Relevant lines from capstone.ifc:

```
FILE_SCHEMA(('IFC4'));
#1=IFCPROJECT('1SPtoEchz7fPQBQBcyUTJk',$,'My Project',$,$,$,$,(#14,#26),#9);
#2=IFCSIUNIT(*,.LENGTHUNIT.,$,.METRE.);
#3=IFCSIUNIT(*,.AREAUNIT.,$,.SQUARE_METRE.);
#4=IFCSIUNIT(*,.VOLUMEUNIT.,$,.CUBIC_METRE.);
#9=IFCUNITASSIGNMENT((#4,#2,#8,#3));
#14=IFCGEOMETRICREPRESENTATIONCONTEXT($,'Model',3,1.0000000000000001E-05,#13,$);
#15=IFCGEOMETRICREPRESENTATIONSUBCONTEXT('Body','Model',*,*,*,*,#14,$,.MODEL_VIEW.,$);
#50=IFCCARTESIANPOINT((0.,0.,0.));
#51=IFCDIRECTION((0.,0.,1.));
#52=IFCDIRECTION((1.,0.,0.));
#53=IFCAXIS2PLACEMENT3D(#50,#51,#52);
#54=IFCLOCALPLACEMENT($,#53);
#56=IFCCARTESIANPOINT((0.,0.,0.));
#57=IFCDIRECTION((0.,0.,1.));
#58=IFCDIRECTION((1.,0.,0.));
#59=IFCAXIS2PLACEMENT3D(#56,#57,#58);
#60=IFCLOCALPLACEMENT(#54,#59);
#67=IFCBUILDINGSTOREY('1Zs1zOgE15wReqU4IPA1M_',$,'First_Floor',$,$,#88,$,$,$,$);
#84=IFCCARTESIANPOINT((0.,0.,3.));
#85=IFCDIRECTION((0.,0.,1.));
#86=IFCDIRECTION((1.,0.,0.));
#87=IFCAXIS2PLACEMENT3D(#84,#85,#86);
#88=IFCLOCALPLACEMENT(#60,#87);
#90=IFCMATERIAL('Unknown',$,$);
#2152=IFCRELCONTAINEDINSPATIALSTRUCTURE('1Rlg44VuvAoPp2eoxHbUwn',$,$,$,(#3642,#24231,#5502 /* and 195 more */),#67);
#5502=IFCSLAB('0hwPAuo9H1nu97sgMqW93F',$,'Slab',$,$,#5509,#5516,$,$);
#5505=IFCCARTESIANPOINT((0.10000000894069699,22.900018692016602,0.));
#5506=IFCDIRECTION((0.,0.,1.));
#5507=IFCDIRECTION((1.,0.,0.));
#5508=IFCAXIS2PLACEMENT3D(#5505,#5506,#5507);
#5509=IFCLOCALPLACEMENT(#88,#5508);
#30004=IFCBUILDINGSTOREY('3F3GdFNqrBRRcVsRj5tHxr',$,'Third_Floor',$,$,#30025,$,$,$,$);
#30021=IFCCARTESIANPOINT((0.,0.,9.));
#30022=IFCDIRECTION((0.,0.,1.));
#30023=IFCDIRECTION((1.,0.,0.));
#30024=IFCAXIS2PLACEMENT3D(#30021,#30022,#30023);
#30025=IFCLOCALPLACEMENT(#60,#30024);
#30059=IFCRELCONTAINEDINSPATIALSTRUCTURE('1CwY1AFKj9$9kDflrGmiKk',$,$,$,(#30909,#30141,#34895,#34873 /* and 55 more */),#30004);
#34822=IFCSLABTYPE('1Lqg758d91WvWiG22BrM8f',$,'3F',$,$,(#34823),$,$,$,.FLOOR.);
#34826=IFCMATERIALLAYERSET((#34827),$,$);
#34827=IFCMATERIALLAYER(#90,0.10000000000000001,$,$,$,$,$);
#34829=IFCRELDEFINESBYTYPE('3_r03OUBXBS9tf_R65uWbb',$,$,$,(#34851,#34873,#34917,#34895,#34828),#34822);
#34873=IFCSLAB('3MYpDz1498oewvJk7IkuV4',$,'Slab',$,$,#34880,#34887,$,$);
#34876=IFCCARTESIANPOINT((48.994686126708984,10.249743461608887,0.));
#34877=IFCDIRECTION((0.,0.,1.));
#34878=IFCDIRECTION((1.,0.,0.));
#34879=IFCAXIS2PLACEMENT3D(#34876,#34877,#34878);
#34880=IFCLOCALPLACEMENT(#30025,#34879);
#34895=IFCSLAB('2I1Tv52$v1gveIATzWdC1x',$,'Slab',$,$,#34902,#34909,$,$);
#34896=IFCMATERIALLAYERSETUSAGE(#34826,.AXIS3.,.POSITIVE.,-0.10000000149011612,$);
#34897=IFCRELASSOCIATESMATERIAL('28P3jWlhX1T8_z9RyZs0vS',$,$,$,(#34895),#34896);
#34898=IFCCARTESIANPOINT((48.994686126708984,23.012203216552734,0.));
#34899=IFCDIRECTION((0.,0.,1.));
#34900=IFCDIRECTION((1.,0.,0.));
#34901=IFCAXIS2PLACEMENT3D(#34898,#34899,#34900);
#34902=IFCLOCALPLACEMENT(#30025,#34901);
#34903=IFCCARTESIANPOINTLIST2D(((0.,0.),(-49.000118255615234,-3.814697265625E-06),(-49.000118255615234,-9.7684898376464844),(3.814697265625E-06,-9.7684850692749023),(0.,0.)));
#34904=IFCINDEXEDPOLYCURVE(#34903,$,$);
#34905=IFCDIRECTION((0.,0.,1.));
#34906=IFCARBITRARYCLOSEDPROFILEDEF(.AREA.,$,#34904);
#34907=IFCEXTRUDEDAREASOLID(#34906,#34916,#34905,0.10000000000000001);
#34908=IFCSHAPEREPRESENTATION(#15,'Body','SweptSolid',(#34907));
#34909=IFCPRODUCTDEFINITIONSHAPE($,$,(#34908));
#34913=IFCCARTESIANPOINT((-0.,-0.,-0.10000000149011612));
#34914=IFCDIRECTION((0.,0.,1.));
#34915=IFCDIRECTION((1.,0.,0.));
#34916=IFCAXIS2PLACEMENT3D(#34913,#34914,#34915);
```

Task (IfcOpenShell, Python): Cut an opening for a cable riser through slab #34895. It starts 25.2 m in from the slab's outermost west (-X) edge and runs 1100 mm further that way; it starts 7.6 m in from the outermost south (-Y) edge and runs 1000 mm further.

```python
import numpy as np
import ifcopenshell
import ifcopenshell.api.feature
import ifcopenshell.api.geometry
import ifcopenshell.api.root
import ifcopenshell.geom
import ifcopenshell.util.placement
import ifcopenshell.util.representation
import ifcopenshell.util.shape
import ifcopenshell.util.unit

model = ifcopenshell.open("capstone.ifc")
unit_scale = ifcopenshell.util.unit.calculate_unit_scale(model)
settings = ifcopenshell.geom.settings()


def volume(element):
    """Net volume in cubic metres, openings subtracted."""
    shape = ifcopenshell.geom.create_shape(settings, element)
    return ifcopenshell.util.shape.get_volume(shape.geometry)


slab = model.by_guid("2I1Tv52$v1gveIATzWdC1x")
before = volume(slab)

# Extent in the slab's own axes, in metres. The edges named are its -X and -Y sides.
slab_shape = ifcopenshell.geom.create_shape(settings, slab)
vertices = ifcopenshell.util.shape.get_vertices(slab_shape.geometry)
x_min, y_min, bottom = vertices.min(axis=0)
top = vertices[:, 2].max()

opening = ifcopenshell.api.root.create_entity(model, ifc_class="IfcOpeningElement", name="Cable riser opening", predefined_type="OPENING")
context = ifcopenshell.util.representation.get_context(model, "Model", "Body", "MODEL_VIEW")
width, depth = 1.1, 1
outline = [(0.0, 0.0), (width, 0.0), (width, depth), (0.0, depth), (0.0, 0.0)]
# Overshoot both faces by 50 mm so the cut is clean.
shape = ifcopenshell.api.geometry.add_slab_representation(
    model, context=context, depth=top - bottom + 0.1, polyline=outline
)
ifcopenshell.api.geometry.assign_representation(model, product=opening, representation=shape)

matrix = ifcopenshell.util.placement.get_local_placement(slab.ObjectPlacement)
matrix[:, 3] = matrix @ np.append(np.array([x_min + 25.2, y_min + 7.6, bottom - 0.05]) / unit_scale, 1.0)
ifcopenshell.api.geometry.edit_object_placement(model, product=opening, matrix=matrix, is_si=False)
ifcopenshell.api.feature.add_feature(model, feature=opening, element=slab)

after = volume(slab)

print(f"slab volume {before:.3f} -> {after:.3f} m3")

model.write("capstone_edited.ifc")
```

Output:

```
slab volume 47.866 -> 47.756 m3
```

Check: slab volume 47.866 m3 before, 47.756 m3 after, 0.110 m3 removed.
